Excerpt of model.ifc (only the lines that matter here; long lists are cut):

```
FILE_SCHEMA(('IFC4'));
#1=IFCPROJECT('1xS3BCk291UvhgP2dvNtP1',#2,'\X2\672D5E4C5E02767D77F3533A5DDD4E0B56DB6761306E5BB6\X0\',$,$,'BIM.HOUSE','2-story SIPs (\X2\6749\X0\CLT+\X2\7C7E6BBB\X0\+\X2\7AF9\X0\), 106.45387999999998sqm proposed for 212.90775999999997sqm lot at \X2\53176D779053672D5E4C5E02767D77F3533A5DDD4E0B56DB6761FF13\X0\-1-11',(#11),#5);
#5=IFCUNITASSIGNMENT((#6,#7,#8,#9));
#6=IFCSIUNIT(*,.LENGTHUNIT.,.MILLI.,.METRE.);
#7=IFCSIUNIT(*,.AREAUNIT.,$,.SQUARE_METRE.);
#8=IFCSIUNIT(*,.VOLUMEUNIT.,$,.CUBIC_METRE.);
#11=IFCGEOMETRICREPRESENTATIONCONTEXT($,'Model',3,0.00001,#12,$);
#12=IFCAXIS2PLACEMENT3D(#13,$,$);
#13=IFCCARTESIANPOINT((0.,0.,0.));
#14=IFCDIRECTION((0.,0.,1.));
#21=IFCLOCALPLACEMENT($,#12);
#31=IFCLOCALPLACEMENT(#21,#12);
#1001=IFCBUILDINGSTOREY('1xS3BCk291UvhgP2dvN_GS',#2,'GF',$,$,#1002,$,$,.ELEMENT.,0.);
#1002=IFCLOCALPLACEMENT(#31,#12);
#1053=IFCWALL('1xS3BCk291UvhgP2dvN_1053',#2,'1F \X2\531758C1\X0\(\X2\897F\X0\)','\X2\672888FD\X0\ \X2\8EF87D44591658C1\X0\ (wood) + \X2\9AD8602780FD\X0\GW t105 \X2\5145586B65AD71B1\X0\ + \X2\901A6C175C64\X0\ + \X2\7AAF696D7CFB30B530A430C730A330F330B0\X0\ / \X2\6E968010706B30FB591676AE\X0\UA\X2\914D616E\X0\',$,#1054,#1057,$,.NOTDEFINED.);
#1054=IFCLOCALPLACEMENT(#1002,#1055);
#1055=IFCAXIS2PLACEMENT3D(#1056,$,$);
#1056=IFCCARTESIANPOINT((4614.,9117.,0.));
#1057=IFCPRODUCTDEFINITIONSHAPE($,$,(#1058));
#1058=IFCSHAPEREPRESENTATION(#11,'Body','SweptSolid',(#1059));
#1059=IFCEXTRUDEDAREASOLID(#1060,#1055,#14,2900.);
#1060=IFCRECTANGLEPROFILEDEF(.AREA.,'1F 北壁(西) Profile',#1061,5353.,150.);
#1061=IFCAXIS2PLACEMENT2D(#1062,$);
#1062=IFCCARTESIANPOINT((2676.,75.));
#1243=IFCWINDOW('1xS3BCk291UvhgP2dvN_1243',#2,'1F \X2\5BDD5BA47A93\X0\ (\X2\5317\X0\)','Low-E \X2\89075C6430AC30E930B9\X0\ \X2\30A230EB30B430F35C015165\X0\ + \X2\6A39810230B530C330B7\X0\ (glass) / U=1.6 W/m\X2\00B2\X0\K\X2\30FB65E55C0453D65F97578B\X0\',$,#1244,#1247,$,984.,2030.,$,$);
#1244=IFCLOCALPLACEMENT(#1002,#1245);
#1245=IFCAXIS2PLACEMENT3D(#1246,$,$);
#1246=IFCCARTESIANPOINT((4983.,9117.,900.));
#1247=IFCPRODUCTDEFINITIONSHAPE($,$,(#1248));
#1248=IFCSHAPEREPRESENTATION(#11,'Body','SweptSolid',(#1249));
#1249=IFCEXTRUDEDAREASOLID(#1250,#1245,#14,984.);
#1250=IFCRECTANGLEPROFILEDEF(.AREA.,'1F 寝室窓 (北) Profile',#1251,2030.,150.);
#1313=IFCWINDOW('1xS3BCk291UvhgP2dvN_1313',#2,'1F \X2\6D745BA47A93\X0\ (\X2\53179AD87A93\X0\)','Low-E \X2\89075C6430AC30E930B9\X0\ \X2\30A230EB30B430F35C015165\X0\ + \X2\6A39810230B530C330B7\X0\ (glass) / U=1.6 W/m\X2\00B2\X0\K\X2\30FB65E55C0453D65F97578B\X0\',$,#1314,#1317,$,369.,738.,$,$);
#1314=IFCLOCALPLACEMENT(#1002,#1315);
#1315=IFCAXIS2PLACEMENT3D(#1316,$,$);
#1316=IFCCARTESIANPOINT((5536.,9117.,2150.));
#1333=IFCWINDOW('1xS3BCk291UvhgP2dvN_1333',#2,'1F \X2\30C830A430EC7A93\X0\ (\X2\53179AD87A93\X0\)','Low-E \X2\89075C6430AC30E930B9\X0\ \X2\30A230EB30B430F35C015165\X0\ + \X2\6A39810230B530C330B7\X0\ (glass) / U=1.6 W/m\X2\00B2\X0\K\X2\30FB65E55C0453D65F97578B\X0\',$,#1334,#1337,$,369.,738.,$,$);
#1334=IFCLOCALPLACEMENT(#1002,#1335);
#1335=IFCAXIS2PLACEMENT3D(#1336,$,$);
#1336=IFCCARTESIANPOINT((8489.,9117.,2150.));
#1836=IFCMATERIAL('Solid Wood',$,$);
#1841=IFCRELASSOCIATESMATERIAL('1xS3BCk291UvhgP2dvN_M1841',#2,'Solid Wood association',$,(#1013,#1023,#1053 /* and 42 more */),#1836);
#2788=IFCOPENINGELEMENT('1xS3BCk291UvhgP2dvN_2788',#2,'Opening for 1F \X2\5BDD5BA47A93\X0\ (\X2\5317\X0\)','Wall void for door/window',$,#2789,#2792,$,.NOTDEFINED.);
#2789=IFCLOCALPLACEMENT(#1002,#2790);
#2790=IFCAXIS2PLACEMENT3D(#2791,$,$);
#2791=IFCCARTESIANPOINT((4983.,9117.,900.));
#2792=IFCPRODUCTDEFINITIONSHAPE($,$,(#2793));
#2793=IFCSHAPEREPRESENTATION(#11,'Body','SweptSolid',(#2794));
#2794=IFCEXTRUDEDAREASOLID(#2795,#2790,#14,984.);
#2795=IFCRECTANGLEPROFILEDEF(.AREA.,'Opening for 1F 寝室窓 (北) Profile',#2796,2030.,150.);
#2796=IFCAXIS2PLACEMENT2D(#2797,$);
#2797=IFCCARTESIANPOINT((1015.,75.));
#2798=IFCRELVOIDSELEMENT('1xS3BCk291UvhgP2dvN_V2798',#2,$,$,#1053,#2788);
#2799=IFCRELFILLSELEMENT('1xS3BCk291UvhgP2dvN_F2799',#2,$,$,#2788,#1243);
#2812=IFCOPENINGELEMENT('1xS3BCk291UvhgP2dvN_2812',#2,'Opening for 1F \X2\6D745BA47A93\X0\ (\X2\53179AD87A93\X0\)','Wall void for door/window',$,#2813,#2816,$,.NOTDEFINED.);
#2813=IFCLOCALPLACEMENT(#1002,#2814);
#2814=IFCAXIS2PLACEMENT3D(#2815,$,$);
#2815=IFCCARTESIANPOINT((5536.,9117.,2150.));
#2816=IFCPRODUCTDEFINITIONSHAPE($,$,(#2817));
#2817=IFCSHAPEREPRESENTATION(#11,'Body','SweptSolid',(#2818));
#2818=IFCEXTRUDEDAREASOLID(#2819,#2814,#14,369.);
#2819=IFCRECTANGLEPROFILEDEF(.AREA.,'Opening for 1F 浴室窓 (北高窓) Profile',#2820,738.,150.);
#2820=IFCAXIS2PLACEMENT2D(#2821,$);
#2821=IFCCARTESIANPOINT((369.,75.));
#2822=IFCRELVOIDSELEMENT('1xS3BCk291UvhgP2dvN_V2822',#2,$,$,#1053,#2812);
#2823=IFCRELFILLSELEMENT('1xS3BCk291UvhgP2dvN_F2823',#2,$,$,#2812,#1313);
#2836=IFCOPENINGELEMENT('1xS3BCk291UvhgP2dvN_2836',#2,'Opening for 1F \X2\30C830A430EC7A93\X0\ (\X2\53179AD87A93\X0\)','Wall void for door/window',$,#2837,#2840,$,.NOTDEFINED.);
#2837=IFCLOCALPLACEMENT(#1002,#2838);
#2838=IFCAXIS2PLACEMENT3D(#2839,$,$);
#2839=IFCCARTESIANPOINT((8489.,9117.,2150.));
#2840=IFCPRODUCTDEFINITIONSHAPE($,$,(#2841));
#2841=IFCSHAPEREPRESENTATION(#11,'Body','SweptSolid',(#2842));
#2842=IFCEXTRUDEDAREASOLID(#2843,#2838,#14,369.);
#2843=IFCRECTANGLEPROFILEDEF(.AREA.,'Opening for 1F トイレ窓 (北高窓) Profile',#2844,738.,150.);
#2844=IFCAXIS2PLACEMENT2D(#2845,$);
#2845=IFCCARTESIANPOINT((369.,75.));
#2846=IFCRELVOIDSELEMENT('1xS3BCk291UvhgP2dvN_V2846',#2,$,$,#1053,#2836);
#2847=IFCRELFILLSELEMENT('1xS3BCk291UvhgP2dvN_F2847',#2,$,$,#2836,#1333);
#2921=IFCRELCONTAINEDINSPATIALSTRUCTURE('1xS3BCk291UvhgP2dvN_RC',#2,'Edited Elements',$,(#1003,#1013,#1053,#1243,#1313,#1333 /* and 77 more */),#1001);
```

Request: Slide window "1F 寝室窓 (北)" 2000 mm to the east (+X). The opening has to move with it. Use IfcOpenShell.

```python
import ifcopenshell
import ifcopenshell.api.geometry
import ifcopenshell.util.placement
import ifcopenshell.util.unit

model = ifcopenshell.open("model.ifc")
unit_scale = ifcopenshell.util.unit.calculate_unit_scale(model)

window = model.by_guid("1xS3BCk291UvhgP2dvN_1243")
opening = window.FillsVoids[0].RelatingOpeningElement
wall = opening.VoidsElements[0].RelatingBuildingElement

wall_matrix = ifcopenshell.util.placement.get_local_placement(wall.ObjectPlacement)
shift = wall_matrix[:3, 0] * 2 / unit_scale
before = ifcopenshell.util.placement.get_local_placement(window.ObjectPlacement)[:3, 3].copy()

# The window is not placed relative to its opening, so move both.
for product in (opening, window):
    matrix = ifcopenshell.util.placement.get_local_placement(product.ObjectPlacement)
    matrix[:3, 3] += shift
    ifcopenshell.api.geometry.edit_object_placement(model, product=product, matrix=matrix, is_si=False)

after = ifcopenshell.util.placement.get_local_placement(window.ObjectPlacement)[:3, 3]
print("window moved by", (after - before).round(3) + 0.0)

model.write("model_updated.ifc")
```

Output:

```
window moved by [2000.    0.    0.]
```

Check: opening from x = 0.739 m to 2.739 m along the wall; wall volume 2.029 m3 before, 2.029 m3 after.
